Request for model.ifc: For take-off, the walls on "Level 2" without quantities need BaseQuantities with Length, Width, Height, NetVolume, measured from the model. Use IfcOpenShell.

First a look at what the model holds.

```python
import ifcopenshell
import ifcopenshell.util.element
import ifcopenshell.util.unit

model = ifcopenshell.open("model.ifc")
print(model.schema)
for unit_type in ("LENGTHUNIT", "AREAUNIT", "VOLUMEUNIT"):
    print(unit_type, ifcopenshell.util.unit.calculate_unit_scale(model, unit_type))
storey = next(s for s in model.by_type("IfcBuildingStorey") if s.Name == "Level 2")
walls = [e for e in ifcopenshell.util.element.get_decomposition(storey) if e.is_a("IfcWall")]
for e in sorted(walls, key=lambda e: e.id()):
    print(e.id(), e.is_a(), e.Name, list(ifcopenshell.util.element.get_psets(e, qtos_only=True)), sep=" | ")
```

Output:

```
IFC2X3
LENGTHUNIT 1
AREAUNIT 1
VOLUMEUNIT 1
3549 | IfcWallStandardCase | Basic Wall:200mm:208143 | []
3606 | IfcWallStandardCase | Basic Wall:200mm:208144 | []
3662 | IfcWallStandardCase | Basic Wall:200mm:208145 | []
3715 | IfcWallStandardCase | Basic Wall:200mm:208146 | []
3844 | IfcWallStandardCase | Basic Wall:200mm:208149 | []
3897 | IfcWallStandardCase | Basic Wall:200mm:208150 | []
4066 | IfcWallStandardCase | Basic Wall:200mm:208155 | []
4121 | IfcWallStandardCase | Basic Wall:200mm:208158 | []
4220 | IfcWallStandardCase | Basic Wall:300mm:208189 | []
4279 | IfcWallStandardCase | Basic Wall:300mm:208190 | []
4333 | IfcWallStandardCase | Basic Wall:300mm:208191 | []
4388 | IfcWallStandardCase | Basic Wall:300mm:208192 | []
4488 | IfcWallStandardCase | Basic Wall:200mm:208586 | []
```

```python
import ifcopenshell
import ifcopenshell.api.pset
import ifcopenshell.geom
import ifcopenshell.util.element
import ifcopenshell.util.shape
import ifcopenshell.util.unit

model = ifcopenshell.open("model.ifc")
unit_scale = ifcopenshell.util.unit.calculate_unit_scale(model)
volume_scale = ifcopenshell.util.unit.calculate_unit_scale(model, "VOLUMEUNIT")
settings = ifcopenshell.geom.settings()

storey = next(s for s in model.by_type("IfcBuildingStorey") if s.Name == "Level 2")
walls = [e for e in ifcopenshell.util.element.get_decomposition(storey) if e.is_a("IfcWall")]

for e in sorted(walls, key=lambda e: e.id()):
    if ifcopenshell.util.element.get_psets(e, qtos_only=True, should_inherit=False):
        continue
    # Geometry comes back in metres, in the element's own axes.
    shape = ifcopenshell.geom.create_shape(settings, e)
    values = {
        "Length": ifcopenshell.util.shape.get_x(shape.geometry) / unit_scale,
        "Width": ifcopenshell.util.shape.get_y(shape.geometry) / unit_scale,
        "Height": ifcopenshell.util.shape.get_z(shape.geometry) / unit_scale,
        "NetVolume": ifcopenshell.util.shape.get_volume(shape.geometry) / volume_scale,
    }
    qto = ifcopenshell.api.pset.add_qto(model, product=e, name="BaseQuantities")
    ifcopenshell.api.pset.edit_qto(model, qto=qto, properties=values)
    print(e.id(), {k: round(v, 3) for k, v in values.items()})

model.write("model_edited.ifc")
```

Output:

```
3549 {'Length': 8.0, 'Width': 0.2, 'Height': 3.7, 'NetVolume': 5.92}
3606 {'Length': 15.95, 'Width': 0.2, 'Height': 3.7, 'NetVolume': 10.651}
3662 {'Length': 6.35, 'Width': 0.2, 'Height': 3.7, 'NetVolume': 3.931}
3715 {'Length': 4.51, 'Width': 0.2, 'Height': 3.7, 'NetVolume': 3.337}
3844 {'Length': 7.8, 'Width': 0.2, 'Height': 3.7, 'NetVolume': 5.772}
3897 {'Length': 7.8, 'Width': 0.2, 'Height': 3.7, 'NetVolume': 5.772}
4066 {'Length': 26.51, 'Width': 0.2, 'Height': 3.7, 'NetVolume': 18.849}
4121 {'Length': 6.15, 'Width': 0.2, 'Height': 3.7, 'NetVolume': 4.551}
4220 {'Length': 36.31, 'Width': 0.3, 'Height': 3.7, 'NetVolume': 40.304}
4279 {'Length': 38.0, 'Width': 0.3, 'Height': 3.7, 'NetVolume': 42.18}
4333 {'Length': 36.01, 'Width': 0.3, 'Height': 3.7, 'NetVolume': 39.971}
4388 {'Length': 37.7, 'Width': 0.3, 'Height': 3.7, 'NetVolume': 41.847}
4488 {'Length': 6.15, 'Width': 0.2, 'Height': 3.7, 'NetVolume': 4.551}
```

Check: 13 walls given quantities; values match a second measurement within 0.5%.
